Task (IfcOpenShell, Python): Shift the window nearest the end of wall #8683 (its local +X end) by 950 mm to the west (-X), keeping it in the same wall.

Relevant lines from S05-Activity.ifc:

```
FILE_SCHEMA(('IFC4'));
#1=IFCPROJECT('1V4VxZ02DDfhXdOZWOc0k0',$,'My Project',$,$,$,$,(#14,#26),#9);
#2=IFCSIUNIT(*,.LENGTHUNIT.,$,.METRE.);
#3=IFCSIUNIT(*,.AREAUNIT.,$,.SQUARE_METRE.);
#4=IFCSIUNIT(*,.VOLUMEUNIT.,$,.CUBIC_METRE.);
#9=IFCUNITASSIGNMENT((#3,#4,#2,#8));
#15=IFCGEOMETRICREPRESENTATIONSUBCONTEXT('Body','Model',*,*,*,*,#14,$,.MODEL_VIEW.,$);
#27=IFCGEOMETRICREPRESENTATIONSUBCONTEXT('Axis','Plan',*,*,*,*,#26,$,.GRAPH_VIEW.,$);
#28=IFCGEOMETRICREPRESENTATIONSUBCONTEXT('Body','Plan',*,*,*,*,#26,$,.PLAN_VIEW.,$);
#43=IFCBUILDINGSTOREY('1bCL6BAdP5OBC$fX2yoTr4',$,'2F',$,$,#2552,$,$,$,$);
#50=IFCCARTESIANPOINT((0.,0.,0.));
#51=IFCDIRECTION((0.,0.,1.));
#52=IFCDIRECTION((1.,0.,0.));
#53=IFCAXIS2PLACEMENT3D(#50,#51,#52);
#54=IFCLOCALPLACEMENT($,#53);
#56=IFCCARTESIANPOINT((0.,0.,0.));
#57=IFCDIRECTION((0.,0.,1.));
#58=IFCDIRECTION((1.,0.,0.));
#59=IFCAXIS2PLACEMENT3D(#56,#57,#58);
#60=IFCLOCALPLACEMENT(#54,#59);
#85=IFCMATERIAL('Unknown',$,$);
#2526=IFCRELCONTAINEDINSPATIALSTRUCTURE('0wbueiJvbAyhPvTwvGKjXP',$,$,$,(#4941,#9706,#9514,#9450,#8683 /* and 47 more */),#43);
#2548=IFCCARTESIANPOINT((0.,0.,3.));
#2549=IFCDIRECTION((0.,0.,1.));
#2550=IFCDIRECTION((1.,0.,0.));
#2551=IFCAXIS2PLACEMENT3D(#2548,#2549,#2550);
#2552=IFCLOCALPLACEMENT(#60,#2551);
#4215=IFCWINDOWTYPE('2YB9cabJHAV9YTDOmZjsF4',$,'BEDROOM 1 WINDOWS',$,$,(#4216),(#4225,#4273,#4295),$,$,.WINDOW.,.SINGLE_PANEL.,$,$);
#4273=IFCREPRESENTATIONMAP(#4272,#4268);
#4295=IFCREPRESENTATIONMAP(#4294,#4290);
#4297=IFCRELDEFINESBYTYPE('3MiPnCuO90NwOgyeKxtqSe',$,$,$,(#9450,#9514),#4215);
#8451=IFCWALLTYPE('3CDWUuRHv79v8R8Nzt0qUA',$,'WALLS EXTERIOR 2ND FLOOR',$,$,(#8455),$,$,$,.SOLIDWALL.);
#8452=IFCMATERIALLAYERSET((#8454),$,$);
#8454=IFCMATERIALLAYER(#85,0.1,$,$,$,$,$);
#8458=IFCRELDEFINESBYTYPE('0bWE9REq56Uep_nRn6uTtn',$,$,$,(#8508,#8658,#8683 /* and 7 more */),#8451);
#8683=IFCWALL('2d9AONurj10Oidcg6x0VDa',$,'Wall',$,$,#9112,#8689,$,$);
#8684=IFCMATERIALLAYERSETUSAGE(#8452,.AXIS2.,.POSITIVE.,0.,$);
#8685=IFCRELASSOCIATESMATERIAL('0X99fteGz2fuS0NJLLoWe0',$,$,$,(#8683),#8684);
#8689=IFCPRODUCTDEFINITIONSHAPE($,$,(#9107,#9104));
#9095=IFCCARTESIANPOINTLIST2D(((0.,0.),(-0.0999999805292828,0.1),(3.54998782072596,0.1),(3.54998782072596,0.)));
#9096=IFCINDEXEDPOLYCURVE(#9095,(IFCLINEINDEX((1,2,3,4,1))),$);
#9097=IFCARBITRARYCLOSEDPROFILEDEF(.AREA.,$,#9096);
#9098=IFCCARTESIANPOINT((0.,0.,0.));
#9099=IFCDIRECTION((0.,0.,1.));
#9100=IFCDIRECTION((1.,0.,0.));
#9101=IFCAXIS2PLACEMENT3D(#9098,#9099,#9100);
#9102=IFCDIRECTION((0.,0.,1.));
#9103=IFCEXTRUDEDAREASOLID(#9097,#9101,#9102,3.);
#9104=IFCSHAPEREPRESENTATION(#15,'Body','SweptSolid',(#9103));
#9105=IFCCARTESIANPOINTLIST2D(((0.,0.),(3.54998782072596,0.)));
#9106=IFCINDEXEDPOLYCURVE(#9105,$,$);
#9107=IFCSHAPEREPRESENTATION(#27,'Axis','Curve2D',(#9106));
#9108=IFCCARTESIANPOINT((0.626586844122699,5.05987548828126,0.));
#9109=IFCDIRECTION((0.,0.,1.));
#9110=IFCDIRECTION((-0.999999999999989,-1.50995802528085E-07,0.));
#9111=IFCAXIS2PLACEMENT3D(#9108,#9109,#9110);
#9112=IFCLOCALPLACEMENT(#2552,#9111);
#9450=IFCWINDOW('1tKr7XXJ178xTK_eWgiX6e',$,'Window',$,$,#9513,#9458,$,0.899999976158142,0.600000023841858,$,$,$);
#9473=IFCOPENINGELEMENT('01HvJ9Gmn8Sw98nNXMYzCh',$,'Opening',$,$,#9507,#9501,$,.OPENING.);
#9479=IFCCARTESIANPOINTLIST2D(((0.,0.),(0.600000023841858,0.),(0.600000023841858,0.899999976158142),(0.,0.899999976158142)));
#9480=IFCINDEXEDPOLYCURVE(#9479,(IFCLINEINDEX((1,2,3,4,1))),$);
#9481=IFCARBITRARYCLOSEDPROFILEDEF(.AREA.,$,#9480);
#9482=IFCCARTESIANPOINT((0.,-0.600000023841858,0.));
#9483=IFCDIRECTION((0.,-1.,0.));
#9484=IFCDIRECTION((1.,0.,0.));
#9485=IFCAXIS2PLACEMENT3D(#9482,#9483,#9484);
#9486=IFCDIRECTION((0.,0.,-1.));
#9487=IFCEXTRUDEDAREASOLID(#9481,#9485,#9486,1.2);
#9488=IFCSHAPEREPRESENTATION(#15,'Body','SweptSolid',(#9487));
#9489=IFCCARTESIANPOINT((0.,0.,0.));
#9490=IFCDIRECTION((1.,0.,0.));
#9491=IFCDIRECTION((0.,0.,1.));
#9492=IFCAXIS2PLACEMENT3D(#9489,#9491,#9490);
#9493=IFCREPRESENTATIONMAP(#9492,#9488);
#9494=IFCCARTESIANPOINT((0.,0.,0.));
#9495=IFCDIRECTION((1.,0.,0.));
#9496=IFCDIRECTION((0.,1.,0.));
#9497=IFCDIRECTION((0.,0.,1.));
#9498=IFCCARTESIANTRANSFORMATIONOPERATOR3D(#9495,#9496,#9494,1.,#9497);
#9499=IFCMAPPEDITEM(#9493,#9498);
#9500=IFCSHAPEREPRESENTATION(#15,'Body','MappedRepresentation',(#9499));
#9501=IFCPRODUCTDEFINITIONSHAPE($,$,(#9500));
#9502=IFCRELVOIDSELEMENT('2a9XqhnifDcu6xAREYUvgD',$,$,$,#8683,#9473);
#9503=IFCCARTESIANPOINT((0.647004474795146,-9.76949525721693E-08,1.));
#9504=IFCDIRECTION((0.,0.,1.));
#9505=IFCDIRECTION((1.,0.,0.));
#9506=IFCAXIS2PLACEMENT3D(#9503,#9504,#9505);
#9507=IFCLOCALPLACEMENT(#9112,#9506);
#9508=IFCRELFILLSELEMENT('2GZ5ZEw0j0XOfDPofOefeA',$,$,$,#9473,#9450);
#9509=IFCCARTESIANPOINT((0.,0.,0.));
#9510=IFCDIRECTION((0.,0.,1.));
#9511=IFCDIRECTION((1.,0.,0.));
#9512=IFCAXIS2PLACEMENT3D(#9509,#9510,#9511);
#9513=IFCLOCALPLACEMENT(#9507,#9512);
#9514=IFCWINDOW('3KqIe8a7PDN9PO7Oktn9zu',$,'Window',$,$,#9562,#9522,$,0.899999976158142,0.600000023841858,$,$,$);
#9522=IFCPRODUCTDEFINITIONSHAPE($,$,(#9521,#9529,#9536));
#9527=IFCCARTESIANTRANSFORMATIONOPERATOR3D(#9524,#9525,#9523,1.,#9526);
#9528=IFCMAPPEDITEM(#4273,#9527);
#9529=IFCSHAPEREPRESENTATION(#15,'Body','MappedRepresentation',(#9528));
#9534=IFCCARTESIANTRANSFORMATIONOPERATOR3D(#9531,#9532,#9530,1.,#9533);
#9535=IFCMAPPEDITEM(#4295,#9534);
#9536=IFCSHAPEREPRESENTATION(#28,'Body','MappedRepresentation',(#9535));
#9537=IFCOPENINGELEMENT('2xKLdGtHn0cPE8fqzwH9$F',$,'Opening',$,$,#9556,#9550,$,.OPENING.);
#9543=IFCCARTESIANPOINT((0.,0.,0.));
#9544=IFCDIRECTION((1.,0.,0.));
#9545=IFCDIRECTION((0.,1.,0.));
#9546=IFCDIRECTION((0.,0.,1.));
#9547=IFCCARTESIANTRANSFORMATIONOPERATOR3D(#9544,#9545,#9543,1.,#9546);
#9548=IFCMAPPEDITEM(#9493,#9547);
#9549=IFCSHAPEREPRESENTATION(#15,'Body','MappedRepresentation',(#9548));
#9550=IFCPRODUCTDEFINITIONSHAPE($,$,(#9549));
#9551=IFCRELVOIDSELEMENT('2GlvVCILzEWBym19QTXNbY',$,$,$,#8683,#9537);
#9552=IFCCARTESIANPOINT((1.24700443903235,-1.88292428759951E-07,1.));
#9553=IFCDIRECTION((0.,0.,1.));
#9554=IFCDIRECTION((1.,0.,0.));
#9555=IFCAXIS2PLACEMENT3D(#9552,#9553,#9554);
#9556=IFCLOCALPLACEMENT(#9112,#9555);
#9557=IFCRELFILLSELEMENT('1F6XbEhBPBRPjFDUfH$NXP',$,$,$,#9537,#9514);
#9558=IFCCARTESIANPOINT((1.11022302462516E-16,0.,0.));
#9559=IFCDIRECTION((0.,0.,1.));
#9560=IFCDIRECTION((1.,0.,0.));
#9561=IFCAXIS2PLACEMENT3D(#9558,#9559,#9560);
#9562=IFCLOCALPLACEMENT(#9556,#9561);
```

```python
import ifcopenshell
import ifcopenshell.api.geometry
import ifcopenshell.util.placement

model = ifcopenshell.open("S05-Activity.ifc")

window = model.by_guid("3KqIe8a7PDN9PO7Oktn9zu")
opening = window.FillsVoids[0].RelatingOpeningElement
wall = opening.VoidsElements[0].RelatingBuildingElement

wall_matrix = ifcopenshell.util.placement.get_local_placement(wall.ObjectPlacement)
shift = wall_matrix[:3, 0] * 0.95
before = ifcopenshell.util.placement.get_local_placement(window.ObjectPlacement)[:3, 3].copy()

# The window is placed relative to its opening, so it follows when the opening moves.
matrix = ifcopenshell.util.placement.get_local_placement(opening.ObjectPlacement)
matrix[:3, 3] += shift
ifcopenshell.api.geometry.edit_object_placement(
    model, product=opening, matrix=matrix, is_si=False, should_transform_children=True
)

after = ifcopenshell.util.placement.get_local_placement(window.ObjectPlacement)[:3, 3]
print("window moved by", (after - before).round(3) + 0.0)

model.write("S05-Activity_edited.ifc")
```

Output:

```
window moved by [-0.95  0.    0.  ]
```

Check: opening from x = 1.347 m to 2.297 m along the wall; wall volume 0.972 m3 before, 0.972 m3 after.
